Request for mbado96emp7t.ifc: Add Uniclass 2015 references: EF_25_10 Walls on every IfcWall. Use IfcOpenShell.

First a look at what the model holds.

```python
import ifcopenshell

model = ifcopenshell.open("mbado96emp7t.ifc")
print(model.schema)
print("classifications:", [c.Name for c in model.by_type("IfcClassification")])
for ifc_class in ("IfcDoor", "IfcRoof", "IfcStair", "IfcWall", "IfcWindow"):
    print(ifc_class, len(model.by_type(ifc_class)))
```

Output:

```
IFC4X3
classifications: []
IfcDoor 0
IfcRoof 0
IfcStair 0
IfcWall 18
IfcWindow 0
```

```python
import ifcopenshell
import ifcopenshell.api.classification

model = ifcopenshell.open("mbado96emp7t.ifc")

system = ifcopenshell.api.classification.add_classification(model, classification="Uniclass 2015")

codes = {
    "IfcWall": ("EF_25_10", "Walls"),
}
for ifc_class, (code, name) in codes.items():
    products = model.by_type(ifc_class)
    ifcopenshell.api.classification.add_reference(
        model, products=products, classification=system, identification=code, name=name
    )
    print(code, len(products))

model.write("mbado96emp7t_rev.ifc")
```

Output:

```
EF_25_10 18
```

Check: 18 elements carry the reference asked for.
